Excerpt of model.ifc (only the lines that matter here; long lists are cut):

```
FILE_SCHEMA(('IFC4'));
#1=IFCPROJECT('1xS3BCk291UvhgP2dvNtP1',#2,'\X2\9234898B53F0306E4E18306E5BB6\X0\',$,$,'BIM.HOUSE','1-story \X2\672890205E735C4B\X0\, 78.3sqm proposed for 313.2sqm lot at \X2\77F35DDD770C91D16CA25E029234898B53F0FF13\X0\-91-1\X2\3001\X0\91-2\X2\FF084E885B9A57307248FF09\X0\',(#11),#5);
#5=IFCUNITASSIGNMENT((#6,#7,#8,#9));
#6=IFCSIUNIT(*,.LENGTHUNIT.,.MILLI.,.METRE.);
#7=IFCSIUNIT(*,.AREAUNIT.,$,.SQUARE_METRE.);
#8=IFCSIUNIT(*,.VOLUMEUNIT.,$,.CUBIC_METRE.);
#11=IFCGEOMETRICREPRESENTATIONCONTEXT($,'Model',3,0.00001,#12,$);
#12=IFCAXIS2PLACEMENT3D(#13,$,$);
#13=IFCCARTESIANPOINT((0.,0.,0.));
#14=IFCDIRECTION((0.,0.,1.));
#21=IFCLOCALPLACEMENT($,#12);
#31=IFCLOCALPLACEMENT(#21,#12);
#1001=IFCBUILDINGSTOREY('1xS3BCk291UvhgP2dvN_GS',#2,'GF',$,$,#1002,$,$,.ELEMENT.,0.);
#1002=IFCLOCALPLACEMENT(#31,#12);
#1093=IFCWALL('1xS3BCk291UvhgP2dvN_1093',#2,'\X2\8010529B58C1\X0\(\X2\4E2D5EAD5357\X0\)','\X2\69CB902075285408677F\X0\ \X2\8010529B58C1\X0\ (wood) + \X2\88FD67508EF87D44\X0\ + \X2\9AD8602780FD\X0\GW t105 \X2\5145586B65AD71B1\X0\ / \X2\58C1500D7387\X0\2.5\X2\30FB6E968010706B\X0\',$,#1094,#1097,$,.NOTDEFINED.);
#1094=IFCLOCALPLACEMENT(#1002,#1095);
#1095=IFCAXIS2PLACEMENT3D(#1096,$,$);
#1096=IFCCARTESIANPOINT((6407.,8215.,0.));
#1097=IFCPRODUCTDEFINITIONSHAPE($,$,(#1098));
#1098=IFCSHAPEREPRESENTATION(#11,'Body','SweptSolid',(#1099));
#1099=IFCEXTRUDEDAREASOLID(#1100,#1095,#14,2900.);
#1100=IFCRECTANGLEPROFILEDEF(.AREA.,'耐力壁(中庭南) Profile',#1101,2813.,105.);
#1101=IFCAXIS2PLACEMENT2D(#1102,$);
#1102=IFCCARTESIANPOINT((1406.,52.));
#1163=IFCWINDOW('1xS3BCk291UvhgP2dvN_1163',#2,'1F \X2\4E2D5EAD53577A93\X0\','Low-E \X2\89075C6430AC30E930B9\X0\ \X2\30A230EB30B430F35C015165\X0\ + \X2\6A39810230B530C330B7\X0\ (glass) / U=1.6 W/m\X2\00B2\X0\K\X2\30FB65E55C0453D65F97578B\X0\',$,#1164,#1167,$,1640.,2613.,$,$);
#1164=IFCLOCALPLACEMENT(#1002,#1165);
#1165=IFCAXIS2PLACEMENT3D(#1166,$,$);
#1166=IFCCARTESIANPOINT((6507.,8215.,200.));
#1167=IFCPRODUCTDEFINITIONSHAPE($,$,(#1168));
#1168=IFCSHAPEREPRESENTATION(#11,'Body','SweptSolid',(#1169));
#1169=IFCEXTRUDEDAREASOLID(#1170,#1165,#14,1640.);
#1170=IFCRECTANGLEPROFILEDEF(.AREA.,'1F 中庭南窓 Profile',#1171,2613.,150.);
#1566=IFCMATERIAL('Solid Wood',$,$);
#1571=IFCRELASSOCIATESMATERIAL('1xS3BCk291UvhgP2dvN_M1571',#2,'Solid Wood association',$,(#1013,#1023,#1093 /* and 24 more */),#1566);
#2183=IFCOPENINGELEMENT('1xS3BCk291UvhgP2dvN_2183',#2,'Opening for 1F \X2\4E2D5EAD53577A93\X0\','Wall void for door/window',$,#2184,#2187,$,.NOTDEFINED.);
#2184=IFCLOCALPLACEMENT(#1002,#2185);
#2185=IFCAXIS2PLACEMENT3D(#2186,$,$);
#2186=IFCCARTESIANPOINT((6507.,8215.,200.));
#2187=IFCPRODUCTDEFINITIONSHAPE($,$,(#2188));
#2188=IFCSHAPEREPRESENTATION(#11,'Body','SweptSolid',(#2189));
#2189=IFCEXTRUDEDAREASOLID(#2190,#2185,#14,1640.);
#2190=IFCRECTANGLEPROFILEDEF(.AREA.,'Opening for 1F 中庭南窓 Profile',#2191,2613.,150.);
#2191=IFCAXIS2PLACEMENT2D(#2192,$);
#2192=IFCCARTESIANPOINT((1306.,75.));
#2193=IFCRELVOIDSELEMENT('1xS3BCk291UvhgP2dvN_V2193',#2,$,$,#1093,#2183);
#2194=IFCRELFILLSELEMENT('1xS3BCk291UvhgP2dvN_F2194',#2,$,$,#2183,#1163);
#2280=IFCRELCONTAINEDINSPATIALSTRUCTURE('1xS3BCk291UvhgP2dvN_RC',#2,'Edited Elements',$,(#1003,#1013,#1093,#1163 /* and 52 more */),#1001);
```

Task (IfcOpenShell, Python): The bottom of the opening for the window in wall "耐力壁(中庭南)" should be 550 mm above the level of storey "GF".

```python
import numpy as np
import ifcopenshell
import ifcopenshell.api.geometry
import ifcopenshell.geom
import ifcopenshell.util.element
import ifcopenshell.util.placement
import ifcopenshell.util.shape
import ifcopenshell.util.unit

model = ifcopenshell.open("model.ifc")
unit_scale = ifcopenshell.util.unit.calculate_unit_scale(model)

window = model.by_guid("1xS3BCk291UvhgP2dvN_1163")
opening = window.FillsVoids[0].RelatingOpeningElement
storey = ifcopenshell.util.element.get_container(window, ifc_class="IfcBuildingStorey")
level = ifcopenshell.util.placement.get_local_placement(storey.ObjectPlacement)[2, 3]

# The opening's origin need not be at the sill, so measure its lowest point.
shape = ifcopenshell.geom.create_shape(ifcopenshell.geom.settings(), opening)
bottom = ifcopenshell.util.shape.get_shape_bottom_elevation(shape, shape.geometry) / unit_scale
dz = level + 0.55 / unit_scale - bottom

shift = np.array([0.0, 0.0, dz])
# The window is not placed relative to its opening, so move both.
for product in (opening, window):
    matrix = ifcopenshell.util.placement.get_local_placement(product.ObjectPlacement)
    matrix[:3, 3] += shift
    ifcopenshell.api.geometry.edit_object_placement(model, product=product, matrix=matrix, is_si=False)

print(f"moved by {dz * unit_scale:+.3f} m")

model.write("model_updated.ifc")
```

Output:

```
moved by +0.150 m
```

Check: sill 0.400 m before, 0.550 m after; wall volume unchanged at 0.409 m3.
